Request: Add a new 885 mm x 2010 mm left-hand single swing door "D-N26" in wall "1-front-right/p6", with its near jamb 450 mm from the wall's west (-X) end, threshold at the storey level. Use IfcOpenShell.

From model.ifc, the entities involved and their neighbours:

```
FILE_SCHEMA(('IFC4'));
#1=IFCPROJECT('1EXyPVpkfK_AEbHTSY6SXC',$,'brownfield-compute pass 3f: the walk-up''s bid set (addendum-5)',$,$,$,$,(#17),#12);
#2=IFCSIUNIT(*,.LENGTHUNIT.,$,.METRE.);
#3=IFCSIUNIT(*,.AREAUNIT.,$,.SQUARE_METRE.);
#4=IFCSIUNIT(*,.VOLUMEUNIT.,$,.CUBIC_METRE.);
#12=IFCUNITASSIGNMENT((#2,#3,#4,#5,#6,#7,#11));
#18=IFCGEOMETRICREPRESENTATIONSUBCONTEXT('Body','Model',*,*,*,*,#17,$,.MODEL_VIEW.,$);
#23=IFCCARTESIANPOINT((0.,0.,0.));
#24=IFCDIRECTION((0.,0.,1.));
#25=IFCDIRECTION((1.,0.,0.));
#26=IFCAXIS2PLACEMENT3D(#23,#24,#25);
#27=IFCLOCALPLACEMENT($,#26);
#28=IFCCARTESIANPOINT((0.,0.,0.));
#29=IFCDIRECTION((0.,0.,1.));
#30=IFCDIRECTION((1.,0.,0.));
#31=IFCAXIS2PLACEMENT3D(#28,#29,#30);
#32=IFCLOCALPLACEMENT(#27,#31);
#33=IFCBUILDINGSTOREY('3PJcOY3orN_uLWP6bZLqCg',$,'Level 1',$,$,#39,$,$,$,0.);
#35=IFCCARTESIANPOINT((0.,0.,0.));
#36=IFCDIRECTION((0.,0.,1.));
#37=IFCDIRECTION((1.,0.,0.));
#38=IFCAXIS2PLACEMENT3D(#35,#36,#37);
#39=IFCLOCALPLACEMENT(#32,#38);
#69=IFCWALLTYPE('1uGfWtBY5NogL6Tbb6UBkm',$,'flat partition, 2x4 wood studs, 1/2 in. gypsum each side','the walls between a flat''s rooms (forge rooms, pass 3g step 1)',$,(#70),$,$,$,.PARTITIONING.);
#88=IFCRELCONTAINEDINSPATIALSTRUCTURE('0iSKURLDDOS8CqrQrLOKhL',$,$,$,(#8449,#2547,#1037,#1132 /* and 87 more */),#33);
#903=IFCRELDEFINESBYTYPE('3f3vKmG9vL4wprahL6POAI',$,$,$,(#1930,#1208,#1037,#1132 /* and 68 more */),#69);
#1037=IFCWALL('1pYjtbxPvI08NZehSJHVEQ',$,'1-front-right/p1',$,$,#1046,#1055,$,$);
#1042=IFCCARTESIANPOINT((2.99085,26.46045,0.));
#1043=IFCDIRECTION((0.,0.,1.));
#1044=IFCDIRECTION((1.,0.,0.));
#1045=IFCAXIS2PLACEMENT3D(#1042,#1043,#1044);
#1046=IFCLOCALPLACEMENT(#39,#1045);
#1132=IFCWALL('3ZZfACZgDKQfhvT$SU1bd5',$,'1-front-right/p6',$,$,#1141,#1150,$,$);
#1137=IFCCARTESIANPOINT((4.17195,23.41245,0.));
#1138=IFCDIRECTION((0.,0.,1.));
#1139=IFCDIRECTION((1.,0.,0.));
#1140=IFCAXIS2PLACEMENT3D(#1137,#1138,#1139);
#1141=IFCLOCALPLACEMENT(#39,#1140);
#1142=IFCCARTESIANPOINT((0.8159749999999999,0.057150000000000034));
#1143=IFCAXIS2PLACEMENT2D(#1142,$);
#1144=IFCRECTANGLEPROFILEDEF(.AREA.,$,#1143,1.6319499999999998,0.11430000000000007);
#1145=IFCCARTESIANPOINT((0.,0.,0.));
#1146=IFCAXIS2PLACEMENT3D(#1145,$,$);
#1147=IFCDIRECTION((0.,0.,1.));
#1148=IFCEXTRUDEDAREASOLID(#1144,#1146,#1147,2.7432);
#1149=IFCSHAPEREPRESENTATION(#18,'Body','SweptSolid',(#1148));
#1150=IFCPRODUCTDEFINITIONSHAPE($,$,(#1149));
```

```python
import numpy as np
import ifcopenshell
import ifcopenshell.api.feature
import ifcopenshell.api.geometry
import ifcopenshell.api.root
import ifcopenshell.api.spatial
import ifcopenshell.geom
import ifcopenshell.util.element
import ifcopenshell.util.placement
import ifcopenshell.util.representation
import ifcopenshell.util.shape
import ifcopenshell.util.unit

model = ifcopenshell.open("model.ifc")
unit_scale = ifcopenshell.util.unit.calculate_unit_scale(model)
settings = ifcopenshell.geom.settings()


def volume(element):
    """Net volume in cubic metres, openings subtracted."""
    shape = ifcopenshell.geom.create_shape(settings, element)
    return ifcopenshell.util.shape.get_volume(shape.geometry)


wall = model.by_guid("3ZZfACZgDKQfhvT$SU1bd5")
storey = ifcopenshell.util.element.get_container(wall, ifc_class="IfcBuildingStorey")
context = ifcopenshell.util.representation.get_context(model, "Model", "Body", "MODEL_VIEW")
before = volume(wall)

width, height, from_end, sill = 0.885, 2.01, 0.45, 0.0  # metres

# The wall runs along its own X axis, and the end named is its -X end.
wall_shape = ifcopenshell.geom.create_shape(settings, wall)
x, y, z = ifcopenshell.util.shape.get_vertices(wall_shape.geometry).T
start = x.min() + from_end
face, thickness = float(y.min()), float(y.max() - y.min())
wall_matrix = ifcopenshell.util.placement.get_local_placement(wall.ObjectPlacement)
level = ifcopenshell.util.placement.get_local_placement(storey.ObjectPlacement)[2, 3]


def in_wall(x, y):
    """Placement at x, y metres in the wall's axes, at sill height."""
    matrix = wall_matrix.copy()
    matrix[:, 3] = wall_matrix @ np.array([x / unit_scale, y / unit_scale, 0.0, 1.0])
    matrix[2, 3] = level + sill / unit_scale
    return matrix


# Opening: a box that overshoots both wall faces by 50 mm.
opening = ifcopenshell.api.root.create_entity(model, ifc_class="IfcOpeningElement", predefined_type="OPENING")
box = ifcopenshell.api.geometry.add_wall_representation(
    model, context=context, length=width, height=height, thickness=thickness + 0.1
)
ifcopenshell.api.geometry.assign_representation(model, product=opening, representation=box)
ifcopenshell.api.geometry.edit_object_placement(model, product=opening, matrix=in_wall(start, face - 0.05), is_si=False)
ifcopenshell.api.feature.add_feature(model, feature=opening, element=wall)

door = ifcopenshell.api.root.create_entity(model, ifc_class="IfcDoor", name="D-N26", predefined_type="DOOR")
door.OverallWidth, door.OverallHeight = width / unit_scale, height / unit_scale
door.OperationType = "SINGLE_SWING_LEFT"
body = ifcopenshell.api.geometry.add_door_representation(
    model,
    context=context,
    overall_width=door.OverallWidth,
    overall_height=door.OverallHeight,
    operation_type="SINGLE_SWING_LEFT",
    lining_properties={"LiningDepth": thickness / unit_scale, "ThresholdDepth": thickness / unit_scale},
)
ifcopenshell.api.geometry.assign_representation(model, product=door, representation=body)
ifcopenshell.api.spatial.assign_container(model, products=[door], relating_structure=storey)
ifcopenshell.api.feature.add_filling(model, opening=opening, element=door)

# The lining spans the wall, so the door starts at the wall face.
ifcopenshell.api.geometry.edit_object_placement(model, product=door, matrix=in_wall(start, face), is_si=False)

after = volume(wall)

print(f"wall volume {before:.3f} -> {after:.3f} m3")

model.write("model-out.ifc")
```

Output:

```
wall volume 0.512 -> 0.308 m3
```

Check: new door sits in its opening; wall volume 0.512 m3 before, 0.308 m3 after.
